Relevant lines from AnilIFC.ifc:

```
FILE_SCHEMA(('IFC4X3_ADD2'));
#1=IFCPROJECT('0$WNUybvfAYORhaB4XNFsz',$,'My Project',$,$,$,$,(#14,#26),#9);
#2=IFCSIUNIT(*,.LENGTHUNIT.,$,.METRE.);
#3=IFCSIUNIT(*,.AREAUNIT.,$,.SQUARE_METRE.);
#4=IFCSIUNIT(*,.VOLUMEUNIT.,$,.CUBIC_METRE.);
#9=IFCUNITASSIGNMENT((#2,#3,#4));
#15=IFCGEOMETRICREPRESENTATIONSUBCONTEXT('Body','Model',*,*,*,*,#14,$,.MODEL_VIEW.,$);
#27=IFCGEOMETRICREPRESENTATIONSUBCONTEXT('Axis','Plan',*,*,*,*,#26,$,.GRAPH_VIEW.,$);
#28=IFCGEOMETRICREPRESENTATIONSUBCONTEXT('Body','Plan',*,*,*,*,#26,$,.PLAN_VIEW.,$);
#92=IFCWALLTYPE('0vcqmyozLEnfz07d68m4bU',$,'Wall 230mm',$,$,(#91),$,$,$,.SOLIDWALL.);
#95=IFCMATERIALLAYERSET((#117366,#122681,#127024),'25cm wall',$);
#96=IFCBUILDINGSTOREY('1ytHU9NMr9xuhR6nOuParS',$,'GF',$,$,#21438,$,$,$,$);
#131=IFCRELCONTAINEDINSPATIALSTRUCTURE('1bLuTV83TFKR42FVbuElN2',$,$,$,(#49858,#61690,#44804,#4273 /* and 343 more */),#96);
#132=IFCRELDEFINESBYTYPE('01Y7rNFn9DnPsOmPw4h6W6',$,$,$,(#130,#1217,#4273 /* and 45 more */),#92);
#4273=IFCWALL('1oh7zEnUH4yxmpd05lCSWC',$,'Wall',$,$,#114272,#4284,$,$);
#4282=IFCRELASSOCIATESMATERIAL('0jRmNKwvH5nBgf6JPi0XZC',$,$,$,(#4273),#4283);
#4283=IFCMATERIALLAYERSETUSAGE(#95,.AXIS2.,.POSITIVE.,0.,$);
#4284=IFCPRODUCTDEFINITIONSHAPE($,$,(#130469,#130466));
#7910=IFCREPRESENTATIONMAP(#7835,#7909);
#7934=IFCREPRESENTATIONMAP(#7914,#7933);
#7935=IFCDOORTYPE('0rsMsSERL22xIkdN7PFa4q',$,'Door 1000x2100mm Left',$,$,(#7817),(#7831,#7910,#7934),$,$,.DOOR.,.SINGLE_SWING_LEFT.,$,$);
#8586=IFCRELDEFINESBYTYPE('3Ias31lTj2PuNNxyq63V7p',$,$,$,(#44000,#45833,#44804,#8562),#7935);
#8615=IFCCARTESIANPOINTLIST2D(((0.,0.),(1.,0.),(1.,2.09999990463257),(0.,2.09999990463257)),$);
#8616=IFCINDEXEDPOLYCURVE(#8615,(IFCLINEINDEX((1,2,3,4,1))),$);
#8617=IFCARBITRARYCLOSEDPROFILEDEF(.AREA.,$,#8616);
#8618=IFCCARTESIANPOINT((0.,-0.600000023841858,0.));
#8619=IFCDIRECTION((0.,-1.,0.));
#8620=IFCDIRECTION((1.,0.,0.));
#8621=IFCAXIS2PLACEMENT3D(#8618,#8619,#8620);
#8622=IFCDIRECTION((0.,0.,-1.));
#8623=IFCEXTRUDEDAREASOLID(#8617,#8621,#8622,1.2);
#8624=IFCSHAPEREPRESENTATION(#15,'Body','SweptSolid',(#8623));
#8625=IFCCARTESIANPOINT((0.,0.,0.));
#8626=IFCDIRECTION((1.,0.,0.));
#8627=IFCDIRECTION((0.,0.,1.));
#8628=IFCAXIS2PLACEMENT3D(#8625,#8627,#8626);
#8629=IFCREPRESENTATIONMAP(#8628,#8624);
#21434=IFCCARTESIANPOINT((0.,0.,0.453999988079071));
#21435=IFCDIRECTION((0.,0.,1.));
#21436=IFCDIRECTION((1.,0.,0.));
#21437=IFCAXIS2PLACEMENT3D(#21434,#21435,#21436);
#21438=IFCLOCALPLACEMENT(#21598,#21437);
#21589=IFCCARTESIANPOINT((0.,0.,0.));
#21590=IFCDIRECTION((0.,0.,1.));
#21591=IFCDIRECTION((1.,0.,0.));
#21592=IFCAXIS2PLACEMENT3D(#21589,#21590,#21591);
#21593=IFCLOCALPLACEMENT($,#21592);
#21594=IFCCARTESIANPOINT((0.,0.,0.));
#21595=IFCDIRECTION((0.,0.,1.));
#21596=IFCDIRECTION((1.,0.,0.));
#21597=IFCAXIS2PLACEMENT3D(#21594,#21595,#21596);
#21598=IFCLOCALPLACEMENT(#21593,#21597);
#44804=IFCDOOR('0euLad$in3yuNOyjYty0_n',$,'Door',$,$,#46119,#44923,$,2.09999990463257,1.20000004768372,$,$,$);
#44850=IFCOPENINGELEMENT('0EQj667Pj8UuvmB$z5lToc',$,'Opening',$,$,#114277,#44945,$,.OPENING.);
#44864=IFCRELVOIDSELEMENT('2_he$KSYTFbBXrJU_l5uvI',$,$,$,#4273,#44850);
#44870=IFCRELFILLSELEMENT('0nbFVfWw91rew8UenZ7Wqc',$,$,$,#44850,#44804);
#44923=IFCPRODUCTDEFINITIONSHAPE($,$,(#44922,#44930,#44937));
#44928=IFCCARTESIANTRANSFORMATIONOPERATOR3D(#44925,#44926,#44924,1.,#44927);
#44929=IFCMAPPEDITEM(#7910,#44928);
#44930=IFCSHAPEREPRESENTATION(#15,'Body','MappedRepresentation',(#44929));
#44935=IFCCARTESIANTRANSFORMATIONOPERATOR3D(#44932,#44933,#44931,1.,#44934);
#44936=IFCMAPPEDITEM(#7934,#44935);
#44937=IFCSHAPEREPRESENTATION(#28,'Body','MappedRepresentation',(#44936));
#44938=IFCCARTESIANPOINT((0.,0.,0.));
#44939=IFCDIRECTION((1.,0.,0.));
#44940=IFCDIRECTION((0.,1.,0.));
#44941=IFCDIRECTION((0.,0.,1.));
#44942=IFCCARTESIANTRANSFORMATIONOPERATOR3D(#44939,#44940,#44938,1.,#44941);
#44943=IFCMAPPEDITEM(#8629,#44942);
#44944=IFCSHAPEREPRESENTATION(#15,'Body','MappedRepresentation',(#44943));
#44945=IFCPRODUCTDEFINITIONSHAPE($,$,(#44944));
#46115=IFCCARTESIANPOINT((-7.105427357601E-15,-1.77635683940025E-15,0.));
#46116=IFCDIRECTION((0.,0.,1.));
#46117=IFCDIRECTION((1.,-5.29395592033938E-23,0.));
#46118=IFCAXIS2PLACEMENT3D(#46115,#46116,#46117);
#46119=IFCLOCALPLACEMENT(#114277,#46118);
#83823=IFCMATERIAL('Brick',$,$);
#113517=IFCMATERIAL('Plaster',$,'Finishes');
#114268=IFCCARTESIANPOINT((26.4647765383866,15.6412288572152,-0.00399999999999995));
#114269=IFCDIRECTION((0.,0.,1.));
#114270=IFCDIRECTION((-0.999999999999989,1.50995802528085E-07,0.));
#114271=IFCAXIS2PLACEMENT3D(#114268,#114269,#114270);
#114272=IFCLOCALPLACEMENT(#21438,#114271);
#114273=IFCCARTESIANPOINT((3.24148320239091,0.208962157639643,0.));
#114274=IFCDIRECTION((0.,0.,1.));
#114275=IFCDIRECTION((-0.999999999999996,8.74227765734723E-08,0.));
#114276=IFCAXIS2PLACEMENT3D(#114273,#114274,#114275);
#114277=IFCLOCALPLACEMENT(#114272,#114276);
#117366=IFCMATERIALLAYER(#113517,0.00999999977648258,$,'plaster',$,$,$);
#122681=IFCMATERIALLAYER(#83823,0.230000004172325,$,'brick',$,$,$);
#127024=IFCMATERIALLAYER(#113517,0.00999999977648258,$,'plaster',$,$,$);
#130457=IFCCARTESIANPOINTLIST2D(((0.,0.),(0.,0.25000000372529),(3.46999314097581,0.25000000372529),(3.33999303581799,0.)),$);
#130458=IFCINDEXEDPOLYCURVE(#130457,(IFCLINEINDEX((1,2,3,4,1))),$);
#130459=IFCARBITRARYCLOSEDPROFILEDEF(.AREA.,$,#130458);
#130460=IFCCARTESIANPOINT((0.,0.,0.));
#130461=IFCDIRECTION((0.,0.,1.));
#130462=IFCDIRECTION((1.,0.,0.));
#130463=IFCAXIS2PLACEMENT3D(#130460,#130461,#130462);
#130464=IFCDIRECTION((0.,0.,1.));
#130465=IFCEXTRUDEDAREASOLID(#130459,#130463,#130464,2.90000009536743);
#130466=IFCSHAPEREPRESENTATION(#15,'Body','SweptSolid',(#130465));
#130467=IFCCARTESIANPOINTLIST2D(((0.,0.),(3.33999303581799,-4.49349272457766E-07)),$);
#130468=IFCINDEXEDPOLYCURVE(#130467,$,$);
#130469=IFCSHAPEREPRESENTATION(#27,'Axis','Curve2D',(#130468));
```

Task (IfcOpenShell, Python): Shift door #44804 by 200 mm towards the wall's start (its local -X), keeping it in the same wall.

```python
import ifcopenshell
import ifcopenshell.api.geometry
import ifcopenshell.util.placement
import ifcopenshell.util.unit

model = ifcopenshell.open("AnilIFC.ifc")
unit_scale = ifcopenshell.util.unit.calculate_unit_scale(model)

door = model.by_id(44804)
opening = door.FillsVoids[0].RelatingOpeningElement
wall = opening.VoidsElements[0].RelatingBuildingElement

wall_matrix = ifcopenshell.util.placement.get_local_placement(wall.ObjectPlacement)
shift = wall_matrix[:3, 0] * -0.2 / unit_scale
before = ifcopenshell.util.placement.get_local_placement(door.ObjectPlacement)[:3, 3].copy()

# The door is placed relative to its opening, so it follows when the opening moves.
matrix = ifcopenshell.util.placement.get_local_placement(opening.ObjectPlacement)
matrix[:3, 3] += shift
ifcopenshell.api.geometry.edit_object_placement(
    model, product=opening, matrix=matrix, is_si=False, should_transform_children=True
)

after = ifcopenshell.util.placement.get_local_placement(door.ObjectPlacement)[:3, 3]
print("door moved by", (after - before).round(3) + 0.0)

model.write("AnilIFC_edited.ifc")
```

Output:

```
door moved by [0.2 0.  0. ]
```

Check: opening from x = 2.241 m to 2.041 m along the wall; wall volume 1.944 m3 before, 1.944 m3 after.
